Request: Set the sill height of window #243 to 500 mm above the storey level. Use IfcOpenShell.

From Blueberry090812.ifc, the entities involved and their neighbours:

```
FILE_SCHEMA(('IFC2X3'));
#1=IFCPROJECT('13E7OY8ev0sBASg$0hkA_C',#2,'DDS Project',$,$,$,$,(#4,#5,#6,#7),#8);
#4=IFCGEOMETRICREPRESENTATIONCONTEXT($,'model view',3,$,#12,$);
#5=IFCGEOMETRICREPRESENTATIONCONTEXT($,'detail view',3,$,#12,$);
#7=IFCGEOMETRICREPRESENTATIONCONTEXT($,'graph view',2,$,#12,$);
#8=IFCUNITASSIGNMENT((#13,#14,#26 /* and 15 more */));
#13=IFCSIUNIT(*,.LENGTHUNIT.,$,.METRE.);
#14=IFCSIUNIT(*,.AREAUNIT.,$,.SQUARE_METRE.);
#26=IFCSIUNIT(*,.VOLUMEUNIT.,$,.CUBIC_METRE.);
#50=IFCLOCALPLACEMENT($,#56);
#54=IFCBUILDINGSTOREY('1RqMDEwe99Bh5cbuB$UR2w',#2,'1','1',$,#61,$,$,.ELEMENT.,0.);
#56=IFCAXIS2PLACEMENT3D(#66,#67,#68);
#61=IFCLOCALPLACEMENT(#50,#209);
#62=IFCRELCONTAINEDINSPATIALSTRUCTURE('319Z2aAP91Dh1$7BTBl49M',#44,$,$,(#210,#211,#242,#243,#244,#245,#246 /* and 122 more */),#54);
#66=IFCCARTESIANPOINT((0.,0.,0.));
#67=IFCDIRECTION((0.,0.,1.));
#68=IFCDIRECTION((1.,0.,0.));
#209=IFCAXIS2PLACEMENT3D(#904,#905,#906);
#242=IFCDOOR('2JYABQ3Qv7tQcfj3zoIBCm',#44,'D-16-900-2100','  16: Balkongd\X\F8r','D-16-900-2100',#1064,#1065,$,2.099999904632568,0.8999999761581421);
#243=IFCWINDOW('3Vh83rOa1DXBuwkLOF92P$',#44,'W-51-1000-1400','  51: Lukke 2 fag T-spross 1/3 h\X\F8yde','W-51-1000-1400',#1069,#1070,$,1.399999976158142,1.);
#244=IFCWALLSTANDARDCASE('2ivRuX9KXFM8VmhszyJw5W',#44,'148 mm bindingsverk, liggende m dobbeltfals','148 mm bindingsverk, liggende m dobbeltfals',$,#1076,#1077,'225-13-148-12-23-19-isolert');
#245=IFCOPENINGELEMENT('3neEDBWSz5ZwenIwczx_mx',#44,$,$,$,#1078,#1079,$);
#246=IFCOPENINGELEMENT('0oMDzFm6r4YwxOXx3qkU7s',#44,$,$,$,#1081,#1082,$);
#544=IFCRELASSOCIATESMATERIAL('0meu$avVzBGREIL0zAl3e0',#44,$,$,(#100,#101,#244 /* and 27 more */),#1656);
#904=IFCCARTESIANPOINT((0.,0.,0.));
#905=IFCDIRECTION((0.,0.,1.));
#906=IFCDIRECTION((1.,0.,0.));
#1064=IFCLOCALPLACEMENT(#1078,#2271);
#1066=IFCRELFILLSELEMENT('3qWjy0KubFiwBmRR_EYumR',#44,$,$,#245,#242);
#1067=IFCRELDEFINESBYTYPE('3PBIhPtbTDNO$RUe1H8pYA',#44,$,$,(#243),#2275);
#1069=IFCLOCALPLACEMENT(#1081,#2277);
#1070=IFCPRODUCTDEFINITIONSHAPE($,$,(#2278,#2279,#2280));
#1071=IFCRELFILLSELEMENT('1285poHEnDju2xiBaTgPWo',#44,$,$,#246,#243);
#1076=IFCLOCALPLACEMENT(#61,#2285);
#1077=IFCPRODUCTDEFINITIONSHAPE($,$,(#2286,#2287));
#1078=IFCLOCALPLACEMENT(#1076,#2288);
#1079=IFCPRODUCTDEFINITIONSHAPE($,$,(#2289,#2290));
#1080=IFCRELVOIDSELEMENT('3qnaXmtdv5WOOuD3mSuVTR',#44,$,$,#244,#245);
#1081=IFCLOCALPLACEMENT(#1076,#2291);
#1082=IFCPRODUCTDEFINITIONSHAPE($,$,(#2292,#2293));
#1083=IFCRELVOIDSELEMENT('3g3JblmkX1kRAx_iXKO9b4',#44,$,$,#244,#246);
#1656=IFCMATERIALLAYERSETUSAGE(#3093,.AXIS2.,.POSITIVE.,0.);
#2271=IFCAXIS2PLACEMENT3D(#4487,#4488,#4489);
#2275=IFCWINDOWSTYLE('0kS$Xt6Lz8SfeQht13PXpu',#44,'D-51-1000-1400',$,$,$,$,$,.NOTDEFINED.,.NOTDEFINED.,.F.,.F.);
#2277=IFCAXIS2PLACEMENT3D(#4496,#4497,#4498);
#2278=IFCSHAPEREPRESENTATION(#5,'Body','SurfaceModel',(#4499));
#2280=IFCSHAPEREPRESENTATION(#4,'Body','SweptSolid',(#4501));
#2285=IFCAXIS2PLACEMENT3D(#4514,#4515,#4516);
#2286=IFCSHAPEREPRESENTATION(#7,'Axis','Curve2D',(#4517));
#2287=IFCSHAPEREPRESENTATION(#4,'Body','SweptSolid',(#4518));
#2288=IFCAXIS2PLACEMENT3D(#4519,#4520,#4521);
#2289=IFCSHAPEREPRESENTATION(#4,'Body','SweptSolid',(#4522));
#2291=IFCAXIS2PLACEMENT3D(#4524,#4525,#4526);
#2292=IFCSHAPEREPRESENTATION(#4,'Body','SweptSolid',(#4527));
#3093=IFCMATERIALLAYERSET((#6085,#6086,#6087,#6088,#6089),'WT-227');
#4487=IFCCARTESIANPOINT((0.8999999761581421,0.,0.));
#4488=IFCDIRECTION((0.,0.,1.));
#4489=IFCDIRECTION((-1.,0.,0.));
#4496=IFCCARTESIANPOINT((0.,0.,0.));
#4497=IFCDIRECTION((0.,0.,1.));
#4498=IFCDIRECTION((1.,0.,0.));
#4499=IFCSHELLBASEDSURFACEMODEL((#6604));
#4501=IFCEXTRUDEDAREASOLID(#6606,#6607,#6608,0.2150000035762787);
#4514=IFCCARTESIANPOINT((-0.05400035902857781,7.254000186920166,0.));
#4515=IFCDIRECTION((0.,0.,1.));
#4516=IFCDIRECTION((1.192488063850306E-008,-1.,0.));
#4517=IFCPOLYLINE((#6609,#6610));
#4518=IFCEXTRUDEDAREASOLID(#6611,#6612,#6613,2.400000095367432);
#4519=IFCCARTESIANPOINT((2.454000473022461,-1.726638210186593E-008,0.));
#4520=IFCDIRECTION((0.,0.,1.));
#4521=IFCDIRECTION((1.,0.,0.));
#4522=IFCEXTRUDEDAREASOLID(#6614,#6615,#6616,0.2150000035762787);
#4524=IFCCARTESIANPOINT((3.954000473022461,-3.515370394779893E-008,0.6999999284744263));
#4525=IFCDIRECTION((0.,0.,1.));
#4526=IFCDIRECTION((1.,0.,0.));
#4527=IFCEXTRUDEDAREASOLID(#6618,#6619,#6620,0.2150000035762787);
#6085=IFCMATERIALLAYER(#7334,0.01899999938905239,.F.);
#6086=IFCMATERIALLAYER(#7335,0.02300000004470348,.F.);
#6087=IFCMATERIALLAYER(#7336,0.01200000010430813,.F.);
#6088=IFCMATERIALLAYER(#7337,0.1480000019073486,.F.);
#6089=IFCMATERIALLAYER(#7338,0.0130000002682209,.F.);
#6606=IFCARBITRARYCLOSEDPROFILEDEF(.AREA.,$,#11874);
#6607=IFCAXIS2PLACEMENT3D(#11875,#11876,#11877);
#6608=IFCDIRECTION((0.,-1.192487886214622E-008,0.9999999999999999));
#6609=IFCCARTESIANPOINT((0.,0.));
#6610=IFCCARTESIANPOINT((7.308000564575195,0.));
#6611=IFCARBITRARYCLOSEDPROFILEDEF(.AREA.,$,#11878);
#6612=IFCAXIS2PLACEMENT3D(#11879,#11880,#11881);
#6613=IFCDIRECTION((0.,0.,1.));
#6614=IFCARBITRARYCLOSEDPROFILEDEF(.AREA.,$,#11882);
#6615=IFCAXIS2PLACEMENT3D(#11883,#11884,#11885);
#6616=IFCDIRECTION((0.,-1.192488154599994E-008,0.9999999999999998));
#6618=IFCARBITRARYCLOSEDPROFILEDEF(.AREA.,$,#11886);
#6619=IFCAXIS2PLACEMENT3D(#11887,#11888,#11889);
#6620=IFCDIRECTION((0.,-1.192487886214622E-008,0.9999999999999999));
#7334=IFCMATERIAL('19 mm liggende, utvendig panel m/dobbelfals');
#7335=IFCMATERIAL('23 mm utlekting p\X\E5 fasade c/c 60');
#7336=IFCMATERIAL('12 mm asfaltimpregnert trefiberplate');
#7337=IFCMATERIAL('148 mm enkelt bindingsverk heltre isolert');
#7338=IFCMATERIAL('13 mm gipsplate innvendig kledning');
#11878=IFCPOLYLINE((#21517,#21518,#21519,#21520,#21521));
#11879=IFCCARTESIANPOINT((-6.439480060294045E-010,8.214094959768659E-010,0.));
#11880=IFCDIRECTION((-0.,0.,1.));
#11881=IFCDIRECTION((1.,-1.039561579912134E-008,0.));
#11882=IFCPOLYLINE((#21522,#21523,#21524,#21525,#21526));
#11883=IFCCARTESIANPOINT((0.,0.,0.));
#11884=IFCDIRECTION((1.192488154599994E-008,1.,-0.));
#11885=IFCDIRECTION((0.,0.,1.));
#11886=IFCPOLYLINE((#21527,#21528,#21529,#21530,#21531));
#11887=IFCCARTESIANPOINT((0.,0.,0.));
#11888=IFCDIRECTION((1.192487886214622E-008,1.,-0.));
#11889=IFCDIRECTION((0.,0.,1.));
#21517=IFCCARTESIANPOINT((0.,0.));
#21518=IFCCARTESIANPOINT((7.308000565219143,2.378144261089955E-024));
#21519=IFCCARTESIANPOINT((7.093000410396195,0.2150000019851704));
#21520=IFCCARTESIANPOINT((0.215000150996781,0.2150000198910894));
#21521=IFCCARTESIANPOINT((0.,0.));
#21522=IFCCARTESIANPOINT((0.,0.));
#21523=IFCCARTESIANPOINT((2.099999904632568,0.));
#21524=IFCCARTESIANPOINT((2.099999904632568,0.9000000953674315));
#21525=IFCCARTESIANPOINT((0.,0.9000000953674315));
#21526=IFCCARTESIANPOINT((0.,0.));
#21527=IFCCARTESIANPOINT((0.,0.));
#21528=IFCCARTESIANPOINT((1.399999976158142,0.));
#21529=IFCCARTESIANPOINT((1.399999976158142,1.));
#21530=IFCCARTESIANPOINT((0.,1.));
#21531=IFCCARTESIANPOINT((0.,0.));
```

```python
import numpy as np
import ifcopenshell
import ifcopenshell.api.geometry
import ifcopenshell.geom
import ifcopenshell.util.element
import ifcopenshell.util.placement
import ifcopenshell.util.shape
import ifcopenshell.util.unit

model = ifcopenshell.open("Blueberry090812.ifc")
unit_scale = ifcopenshell.util.unit.calculate_unit_scale(model)

window = model.by_guid("3Vh83rOa1DXBuwkLOF92P$")
opening = window.FillsVoids[0].RelatingOpeningElement
storey = ifcopenshell.util.element.get_container(window, ifc_class="IfcBuildingStorey")
level = ifcopenshell.util.placement.get_local_placement(storey.ObjectPlacement)[2, 3]

# The opening's origin need not be at the sill, so measure its lowest point.
shape = ifcopenshell.geom.create_shape(ifcopenshell.geom.settings(), opening)
bottom = ifcopenshell.util.shape.get_shape_bottom_elevation(shape, shape.geometry) / unit_scale
dz = level + 0.5 / unit_scale - bottom

shift = np.array([0.0, 0.0, dz])
# The window is placed relative to its opening, so it follows when the opening moves.
matrix = ifcopenshell.util.placement.get_local_placement(opening.ObjectPlacement)
matrix[:3, 3] += shift
ifcopenshell.api.geometry.edit_object_placement(
    model, product=opening, matrix=matrix, is_si=False, should_transform_children=True
)

print(f"moved by {dz * unit_scale:+.3f} m")

model.write("Blueberry090812_edited.ifc")
```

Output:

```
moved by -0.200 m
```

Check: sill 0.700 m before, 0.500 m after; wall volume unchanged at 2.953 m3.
